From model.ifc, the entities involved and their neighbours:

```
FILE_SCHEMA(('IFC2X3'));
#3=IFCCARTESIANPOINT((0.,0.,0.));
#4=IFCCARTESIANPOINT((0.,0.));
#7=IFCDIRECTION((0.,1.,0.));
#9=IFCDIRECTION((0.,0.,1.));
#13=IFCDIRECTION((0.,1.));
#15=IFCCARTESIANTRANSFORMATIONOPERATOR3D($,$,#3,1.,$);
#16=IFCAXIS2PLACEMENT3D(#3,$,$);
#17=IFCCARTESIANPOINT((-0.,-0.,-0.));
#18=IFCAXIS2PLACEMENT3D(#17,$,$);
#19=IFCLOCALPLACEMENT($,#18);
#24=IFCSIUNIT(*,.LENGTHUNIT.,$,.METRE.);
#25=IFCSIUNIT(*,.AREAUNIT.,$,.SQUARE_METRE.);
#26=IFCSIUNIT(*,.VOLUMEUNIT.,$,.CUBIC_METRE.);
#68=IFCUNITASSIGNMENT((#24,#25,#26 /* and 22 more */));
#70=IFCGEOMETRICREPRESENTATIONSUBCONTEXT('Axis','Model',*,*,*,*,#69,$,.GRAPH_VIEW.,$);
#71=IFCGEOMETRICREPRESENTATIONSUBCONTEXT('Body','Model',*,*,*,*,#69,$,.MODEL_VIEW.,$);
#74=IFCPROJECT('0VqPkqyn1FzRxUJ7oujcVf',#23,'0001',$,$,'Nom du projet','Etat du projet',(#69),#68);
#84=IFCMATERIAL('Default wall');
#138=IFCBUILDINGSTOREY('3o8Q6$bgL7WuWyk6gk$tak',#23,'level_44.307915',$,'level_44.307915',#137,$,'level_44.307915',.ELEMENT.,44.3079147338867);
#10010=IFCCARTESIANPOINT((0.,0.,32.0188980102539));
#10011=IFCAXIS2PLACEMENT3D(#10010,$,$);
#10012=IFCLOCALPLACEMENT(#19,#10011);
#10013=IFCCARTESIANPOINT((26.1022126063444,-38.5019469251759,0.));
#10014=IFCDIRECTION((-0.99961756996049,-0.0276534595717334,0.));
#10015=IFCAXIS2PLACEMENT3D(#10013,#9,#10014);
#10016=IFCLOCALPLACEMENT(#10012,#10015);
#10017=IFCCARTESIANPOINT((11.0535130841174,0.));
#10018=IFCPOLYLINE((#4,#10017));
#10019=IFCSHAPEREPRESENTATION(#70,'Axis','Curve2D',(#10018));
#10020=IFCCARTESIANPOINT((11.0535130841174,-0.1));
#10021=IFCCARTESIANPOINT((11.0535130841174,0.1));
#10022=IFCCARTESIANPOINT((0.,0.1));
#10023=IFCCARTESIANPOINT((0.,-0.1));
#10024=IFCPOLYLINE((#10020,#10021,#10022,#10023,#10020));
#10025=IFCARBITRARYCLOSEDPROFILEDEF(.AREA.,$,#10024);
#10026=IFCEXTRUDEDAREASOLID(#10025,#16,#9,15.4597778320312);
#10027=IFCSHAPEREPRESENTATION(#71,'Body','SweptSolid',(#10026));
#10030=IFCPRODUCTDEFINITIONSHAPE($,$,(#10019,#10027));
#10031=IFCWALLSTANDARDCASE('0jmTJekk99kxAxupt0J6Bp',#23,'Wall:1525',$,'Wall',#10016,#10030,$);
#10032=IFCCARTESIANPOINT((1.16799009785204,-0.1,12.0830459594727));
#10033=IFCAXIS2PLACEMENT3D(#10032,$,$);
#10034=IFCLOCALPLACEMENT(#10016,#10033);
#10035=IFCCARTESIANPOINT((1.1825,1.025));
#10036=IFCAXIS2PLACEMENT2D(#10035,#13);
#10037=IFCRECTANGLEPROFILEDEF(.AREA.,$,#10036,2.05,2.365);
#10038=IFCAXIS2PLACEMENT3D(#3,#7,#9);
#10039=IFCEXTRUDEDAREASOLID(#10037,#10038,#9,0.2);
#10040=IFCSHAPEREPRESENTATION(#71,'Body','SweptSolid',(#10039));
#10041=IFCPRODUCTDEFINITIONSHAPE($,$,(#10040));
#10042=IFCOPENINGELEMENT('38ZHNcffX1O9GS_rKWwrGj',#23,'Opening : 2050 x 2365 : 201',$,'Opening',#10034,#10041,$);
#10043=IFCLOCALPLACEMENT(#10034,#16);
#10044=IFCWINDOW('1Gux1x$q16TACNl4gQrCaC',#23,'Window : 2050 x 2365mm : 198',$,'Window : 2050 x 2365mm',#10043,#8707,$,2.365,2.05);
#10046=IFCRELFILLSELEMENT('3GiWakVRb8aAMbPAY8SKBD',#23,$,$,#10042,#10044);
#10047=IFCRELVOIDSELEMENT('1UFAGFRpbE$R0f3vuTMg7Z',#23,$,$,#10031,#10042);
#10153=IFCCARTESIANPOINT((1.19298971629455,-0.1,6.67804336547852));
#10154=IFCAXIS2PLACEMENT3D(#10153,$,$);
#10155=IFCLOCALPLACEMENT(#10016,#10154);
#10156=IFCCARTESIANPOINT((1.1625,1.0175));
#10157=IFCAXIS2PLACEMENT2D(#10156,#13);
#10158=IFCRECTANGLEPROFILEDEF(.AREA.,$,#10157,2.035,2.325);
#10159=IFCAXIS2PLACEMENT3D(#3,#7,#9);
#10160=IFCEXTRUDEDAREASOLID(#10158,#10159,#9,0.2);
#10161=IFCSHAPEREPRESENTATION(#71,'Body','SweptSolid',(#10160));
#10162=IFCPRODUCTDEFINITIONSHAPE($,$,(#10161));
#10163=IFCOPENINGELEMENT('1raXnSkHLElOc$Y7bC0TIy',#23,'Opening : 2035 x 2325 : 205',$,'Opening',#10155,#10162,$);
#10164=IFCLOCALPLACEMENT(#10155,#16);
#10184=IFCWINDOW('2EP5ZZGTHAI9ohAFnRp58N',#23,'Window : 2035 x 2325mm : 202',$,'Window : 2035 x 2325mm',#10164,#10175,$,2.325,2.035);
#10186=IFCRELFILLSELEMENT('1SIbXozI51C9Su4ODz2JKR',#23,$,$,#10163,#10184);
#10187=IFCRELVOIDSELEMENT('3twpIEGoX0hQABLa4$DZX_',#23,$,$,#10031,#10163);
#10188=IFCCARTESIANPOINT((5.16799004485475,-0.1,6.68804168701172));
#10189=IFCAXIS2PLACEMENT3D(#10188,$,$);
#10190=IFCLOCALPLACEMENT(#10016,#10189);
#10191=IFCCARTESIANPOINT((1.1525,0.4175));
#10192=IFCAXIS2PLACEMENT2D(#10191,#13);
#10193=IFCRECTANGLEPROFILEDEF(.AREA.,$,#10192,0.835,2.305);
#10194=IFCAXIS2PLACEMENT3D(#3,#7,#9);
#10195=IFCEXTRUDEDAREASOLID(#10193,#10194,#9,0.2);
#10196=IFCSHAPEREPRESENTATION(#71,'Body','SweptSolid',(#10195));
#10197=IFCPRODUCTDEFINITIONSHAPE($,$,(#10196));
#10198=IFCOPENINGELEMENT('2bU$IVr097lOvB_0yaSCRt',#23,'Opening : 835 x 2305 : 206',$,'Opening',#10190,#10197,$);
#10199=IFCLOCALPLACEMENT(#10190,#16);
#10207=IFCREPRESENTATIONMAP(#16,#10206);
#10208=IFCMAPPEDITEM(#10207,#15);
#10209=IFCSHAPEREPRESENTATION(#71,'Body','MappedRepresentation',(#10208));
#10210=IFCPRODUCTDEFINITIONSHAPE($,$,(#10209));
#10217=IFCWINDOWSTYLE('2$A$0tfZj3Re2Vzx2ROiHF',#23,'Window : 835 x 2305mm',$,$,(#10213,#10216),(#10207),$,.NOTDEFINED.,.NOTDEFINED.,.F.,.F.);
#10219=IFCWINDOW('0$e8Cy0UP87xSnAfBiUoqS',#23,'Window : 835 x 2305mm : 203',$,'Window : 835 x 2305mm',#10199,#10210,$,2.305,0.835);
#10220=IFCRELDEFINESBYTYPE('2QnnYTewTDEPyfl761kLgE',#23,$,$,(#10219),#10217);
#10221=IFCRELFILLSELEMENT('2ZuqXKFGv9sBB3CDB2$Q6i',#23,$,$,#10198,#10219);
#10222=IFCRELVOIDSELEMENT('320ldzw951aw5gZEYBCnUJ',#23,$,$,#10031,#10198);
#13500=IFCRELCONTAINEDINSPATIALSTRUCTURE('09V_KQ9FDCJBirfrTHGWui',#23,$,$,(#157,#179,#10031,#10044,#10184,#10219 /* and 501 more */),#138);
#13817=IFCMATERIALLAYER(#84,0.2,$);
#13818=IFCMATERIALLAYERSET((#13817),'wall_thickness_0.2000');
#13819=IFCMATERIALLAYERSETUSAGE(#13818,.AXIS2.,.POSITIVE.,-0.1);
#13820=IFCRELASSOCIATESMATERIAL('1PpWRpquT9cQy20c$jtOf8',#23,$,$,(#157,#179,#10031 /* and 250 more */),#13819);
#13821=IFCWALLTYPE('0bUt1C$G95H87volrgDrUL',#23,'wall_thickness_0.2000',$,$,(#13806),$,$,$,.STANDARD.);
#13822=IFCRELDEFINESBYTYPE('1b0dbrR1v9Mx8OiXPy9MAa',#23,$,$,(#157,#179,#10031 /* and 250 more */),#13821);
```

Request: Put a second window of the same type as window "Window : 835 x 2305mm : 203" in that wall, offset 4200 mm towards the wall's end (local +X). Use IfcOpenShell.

```python
import ifcopenshell
import ifcopenshell.api.feature
import ifcopenshell.api.geometry
import ifcopenshell.api.root
import ifcopenshell.geom
import ifcopenshell.util.element
import ifcopenshell.util.placement
import ifcopenshell.util.shape

model = ifcopenshell.open("model.ifc")
settings = ifcopenshell.geom.settings()


def volume(element):
    """Net volume in cubic metres, openings subtracted."""
    shape = ifcopenshell.geom.create_shape(settings, element)
    return ifcopenshell.util.shape.get_volume(shape.geometry)


window = model.by_guid("0$e8Cy0UP87xSnAfBiUoqS")
opening = window.FillsVoids[0].RelatingOpeningElement
wall = opening.VoidsElements[0].RelatingBuildingElement
before = volume(wall)
shift = ifcopenshell.util.placement.get_local_placement(wall.ObjectPlacement)[:3, 0] * 4.2

# copy_class copies the void relationship, type, container and properties, but no geometry.
new_opening = ifcopenshell.api.root.copy_class(model, product=opening)
new_opening.Representation = ifcopenshell.util.element.copy_deep(
    model, opening.Representation, exclude=["IfcGeometricRepresentationContext", "IfcRepresentationMap"]
)
new_opening.Name = "Opening : 835 x 2305"
new_window = ifcopenshell.api.root.copy_class(model, product=window)
new_window.Representation = ifcopenshell.util.element.copy_deep(
    model, window.Representation, exclude=["IfcGeometricRepresentationContext", "IfcRepresentationMap"]
)
new_window.Name = "Window : 835 x 2305mm"
fills = ifcopenshell.api.feature.add_filling(model, opening=new_opening, element=new_window)
fills.OwnerHistory = new_window.OwnerHistory  # required in IFC2X3

for old, new in ((opening, new_opening), (window, new_window)):
    matrix = ifcopenshell.util.placement.get_local_placement(old.ObjectPlacement)
    matrix[:3, 3] += shift
    ifcopenshell.api.geometry.edit_object_placement(model, product=new, matrix=matrix, is_si=False)

after = volume(wall)

print(f"wall volume {before:.3f} -> {after:.3f} m3")

model.write("model_edited.ifc")
```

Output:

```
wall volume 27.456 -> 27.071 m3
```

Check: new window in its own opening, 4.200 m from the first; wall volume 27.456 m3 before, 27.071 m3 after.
